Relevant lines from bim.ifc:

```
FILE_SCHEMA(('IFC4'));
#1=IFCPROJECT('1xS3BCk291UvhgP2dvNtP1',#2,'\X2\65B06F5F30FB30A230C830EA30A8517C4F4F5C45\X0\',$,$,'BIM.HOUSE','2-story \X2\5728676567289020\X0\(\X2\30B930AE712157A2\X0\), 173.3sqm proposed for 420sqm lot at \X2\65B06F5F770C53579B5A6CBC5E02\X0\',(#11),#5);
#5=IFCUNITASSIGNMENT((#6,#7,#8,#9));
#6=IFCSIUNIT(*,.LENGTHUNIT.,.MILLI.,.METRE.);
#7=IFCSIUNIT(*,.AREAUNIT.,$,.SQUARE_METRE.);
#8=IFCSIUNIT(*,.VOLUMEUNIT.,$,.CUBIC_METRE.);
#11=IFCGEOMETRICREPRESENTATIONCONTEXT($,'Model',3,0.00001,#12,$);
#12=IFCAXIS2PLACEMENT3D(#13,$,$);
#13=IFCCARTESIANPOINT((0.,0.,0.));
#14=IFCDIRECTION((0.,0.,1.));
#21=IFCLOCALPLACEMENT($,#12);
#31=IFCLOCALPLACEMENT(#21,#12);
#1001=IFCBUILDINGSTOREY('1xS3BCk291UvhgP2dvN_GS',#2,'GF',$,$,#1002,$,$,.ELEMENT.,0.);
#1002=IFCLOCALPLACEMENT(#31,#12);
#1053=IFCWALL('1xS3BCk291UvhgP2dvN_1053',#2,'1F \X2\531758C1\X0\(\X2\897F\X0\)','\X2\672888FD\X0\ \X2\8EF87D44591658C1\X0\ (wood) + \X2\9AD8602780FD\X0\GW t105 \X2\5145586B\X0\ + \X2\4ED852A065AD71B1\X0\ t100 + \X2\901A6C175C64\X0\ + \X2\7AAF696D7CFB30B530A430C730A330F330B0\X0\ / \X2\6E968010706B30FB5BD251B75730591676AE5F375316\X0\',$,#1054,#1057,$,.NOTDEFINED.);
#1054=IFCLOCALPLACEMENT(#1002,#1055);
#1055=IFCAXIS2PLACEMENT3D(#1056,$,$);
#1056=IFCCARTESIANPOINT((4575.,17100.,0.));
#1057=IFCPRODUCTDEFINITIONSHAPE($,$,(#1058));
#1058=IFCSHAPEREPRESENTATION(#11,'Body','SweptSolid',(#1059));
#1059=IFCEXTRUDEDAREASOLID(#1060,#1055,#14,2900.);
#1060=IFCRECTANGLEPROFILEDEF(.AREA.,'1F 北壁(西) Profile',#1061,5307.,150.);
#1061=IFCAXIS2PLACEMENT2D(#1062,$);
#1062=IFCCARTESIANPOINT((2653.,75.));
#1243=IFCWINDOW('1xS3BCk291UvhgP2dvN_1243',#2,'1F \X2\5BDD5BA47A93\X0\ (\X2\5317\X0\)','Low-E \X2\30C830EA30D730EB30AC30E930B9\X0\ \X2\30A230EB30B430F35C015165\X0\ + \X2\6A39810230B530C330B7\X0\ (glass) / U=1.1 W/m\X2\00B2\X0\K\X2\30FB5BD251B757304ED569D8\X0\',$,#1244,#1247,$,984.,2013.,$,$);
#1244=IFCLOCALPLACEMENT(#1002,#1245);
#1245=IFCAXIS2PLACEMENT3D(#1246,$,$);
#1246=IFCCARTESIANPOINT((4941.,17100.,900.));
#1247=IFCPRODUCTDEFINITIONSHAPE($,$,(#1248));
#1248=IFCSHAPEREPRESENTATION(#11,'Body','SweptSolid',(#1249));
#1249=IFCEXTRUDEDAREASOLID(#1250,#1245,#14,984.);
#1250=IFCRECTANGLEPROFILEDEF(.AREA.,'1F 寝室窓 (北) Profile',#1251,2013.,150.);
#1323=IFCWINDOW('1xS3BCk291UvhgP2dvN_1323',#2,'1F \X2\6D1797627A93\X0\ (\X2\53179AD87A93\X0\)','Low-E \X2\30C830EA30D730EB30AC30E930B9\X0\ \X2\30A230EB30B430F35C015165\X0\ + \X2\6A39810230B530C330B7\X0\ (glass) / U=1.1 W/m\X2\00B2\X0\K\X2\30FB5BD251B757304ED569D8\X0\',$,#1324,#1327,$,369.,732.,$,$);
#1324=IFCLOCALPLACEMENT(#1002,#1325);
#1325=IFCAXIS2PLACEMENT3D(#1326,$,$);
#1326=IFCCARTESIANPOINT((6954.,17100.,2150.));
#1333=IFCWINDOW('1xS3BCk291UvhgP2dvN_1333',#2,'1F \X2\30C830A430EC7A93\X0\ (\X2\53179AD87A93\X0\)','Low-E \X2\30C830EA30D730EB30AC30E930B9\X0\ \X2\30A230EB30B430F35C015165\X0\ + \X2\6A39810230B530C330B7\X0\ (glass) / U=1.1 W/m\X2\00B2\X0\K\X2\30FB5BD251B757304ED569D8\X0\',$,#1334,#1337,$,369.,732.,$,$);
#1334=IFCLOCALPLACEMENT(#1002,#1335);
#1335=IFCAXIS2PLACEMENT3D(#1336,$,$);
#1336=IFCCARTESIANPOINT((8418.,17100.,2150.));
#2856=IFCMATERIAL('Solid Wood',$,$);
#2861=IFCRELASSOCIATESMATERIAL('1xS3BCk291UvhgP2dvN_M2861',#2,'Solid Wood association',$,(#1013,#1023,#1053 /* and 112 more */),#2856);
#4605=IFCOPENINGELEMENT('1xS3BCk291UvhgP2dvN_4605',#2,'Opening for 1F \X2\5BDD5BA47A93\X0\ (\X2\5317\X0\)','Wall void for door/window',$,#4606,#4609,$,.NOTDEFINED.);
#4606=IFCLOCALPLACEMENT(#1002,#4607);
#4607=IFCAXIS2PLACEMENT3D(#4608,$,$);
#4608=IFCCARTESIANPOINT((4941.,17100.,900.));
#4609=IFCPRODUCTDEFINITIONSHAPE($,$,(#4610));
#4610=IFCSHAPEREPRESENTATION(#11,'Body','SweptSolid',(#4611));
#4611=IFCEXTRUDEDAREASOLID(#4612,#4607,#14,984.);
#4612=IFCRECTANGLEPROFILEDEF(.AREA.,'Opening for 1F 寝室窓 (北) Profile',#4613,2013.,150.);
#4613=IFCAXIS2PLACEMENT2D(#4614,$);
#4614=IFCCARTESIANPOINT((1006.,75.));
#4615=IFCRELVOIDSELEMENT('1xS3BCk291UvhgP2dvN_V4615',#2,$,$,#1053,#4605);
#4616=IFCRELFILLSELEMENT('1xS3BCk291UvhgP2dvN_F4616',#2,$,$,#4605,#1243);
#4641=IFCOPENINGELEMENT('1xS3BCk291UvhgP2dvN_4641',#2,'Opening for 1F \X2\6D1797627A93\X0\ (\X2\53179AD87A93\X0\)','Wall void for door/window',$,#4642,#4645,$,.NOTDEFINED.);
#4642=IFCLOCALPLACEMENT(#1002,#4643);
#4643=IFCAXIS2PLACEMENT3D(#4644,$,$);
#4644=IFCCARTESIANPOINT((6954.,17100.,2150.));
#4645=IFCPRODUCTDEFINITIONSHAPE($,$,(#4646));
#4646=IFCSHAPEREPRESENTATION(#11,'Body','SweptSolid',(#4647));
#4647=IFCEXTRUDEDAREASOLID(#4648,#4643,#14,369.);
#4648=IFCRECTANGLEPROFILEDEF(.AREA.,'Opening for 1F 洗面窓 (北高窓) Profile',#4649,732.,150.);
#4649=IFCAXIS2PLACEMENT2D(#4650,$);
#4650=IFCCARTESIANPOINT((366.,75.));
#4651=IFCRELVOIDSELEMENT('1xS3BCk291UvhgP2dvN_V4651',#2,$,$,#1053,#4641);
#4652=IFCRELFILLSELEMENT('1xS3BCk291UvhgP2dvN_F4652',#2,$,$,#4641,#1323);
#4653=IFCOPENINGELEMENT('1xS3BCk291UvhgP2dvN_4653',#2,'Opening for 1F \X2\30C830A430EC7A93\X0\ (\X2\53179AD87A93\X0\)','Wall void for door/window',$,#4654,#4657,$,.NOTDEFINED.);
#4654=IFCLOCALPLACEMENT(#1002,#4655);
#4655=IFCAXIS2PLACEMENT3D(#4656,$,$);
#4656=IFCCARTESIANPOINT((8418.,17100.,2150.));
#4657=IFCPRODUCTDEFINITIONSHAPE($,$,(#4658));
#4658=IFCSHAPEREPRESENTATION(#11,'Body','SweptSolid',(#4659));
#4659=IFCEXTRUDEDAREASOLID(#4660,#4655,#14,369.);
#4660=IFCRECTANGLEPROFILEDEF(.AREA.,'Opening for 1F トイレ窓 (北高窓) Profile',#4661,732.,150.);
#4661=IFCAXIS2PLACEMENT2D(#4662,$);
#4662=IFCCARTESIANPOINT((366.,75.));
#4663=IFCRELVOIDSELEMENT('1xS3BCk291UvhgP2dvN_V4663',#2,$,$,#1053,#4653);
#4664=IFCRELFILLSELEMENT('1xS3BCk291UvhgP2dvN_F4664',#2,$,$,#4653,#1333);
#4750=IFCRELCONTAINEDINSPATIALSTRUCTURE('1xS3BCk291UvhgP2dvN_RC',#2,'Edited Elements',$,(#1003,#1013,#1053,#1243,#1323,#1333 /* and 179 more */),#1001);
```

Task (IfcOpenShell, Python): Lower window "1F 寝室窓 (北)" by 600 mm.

```python
import numpy as np
import ifcopenshell
import ifcopenshell.api.geometry
import ifcopenshell.util.placement
import ifcopenshell.util.unit

model = ifcopenshell.open("bim.ifc")
unit_scale = ifcopenshell.util.unit.calculate_unit_scale(model)

window = model.by_guid("1xS3BCk291UvhgP2dvN_1243")
opening = window.FillsVoids[0].RelatingOpeningElement
dz = -0.6 / unit_scale

shift = np.array([0.0, 0.0, dz])
# The window is not placed relative to its opening, so move both.
for product in (opening, window):
    matrix = ifcopenshell.util.placement.get_local_placement(product.ObjectPlacement)
    matrix[:3, 3] += shift
    ifcopenshell.api.geometry.edit_object_placement(model, product=product, matrix=matrix, is_si=False)

print(f"moved by {dz * unit_scale:+.3f} m")

model.write("bim_rev.ifc")
```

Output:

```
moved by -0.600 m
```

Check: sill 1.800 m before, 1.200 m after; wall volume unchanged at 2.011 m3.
